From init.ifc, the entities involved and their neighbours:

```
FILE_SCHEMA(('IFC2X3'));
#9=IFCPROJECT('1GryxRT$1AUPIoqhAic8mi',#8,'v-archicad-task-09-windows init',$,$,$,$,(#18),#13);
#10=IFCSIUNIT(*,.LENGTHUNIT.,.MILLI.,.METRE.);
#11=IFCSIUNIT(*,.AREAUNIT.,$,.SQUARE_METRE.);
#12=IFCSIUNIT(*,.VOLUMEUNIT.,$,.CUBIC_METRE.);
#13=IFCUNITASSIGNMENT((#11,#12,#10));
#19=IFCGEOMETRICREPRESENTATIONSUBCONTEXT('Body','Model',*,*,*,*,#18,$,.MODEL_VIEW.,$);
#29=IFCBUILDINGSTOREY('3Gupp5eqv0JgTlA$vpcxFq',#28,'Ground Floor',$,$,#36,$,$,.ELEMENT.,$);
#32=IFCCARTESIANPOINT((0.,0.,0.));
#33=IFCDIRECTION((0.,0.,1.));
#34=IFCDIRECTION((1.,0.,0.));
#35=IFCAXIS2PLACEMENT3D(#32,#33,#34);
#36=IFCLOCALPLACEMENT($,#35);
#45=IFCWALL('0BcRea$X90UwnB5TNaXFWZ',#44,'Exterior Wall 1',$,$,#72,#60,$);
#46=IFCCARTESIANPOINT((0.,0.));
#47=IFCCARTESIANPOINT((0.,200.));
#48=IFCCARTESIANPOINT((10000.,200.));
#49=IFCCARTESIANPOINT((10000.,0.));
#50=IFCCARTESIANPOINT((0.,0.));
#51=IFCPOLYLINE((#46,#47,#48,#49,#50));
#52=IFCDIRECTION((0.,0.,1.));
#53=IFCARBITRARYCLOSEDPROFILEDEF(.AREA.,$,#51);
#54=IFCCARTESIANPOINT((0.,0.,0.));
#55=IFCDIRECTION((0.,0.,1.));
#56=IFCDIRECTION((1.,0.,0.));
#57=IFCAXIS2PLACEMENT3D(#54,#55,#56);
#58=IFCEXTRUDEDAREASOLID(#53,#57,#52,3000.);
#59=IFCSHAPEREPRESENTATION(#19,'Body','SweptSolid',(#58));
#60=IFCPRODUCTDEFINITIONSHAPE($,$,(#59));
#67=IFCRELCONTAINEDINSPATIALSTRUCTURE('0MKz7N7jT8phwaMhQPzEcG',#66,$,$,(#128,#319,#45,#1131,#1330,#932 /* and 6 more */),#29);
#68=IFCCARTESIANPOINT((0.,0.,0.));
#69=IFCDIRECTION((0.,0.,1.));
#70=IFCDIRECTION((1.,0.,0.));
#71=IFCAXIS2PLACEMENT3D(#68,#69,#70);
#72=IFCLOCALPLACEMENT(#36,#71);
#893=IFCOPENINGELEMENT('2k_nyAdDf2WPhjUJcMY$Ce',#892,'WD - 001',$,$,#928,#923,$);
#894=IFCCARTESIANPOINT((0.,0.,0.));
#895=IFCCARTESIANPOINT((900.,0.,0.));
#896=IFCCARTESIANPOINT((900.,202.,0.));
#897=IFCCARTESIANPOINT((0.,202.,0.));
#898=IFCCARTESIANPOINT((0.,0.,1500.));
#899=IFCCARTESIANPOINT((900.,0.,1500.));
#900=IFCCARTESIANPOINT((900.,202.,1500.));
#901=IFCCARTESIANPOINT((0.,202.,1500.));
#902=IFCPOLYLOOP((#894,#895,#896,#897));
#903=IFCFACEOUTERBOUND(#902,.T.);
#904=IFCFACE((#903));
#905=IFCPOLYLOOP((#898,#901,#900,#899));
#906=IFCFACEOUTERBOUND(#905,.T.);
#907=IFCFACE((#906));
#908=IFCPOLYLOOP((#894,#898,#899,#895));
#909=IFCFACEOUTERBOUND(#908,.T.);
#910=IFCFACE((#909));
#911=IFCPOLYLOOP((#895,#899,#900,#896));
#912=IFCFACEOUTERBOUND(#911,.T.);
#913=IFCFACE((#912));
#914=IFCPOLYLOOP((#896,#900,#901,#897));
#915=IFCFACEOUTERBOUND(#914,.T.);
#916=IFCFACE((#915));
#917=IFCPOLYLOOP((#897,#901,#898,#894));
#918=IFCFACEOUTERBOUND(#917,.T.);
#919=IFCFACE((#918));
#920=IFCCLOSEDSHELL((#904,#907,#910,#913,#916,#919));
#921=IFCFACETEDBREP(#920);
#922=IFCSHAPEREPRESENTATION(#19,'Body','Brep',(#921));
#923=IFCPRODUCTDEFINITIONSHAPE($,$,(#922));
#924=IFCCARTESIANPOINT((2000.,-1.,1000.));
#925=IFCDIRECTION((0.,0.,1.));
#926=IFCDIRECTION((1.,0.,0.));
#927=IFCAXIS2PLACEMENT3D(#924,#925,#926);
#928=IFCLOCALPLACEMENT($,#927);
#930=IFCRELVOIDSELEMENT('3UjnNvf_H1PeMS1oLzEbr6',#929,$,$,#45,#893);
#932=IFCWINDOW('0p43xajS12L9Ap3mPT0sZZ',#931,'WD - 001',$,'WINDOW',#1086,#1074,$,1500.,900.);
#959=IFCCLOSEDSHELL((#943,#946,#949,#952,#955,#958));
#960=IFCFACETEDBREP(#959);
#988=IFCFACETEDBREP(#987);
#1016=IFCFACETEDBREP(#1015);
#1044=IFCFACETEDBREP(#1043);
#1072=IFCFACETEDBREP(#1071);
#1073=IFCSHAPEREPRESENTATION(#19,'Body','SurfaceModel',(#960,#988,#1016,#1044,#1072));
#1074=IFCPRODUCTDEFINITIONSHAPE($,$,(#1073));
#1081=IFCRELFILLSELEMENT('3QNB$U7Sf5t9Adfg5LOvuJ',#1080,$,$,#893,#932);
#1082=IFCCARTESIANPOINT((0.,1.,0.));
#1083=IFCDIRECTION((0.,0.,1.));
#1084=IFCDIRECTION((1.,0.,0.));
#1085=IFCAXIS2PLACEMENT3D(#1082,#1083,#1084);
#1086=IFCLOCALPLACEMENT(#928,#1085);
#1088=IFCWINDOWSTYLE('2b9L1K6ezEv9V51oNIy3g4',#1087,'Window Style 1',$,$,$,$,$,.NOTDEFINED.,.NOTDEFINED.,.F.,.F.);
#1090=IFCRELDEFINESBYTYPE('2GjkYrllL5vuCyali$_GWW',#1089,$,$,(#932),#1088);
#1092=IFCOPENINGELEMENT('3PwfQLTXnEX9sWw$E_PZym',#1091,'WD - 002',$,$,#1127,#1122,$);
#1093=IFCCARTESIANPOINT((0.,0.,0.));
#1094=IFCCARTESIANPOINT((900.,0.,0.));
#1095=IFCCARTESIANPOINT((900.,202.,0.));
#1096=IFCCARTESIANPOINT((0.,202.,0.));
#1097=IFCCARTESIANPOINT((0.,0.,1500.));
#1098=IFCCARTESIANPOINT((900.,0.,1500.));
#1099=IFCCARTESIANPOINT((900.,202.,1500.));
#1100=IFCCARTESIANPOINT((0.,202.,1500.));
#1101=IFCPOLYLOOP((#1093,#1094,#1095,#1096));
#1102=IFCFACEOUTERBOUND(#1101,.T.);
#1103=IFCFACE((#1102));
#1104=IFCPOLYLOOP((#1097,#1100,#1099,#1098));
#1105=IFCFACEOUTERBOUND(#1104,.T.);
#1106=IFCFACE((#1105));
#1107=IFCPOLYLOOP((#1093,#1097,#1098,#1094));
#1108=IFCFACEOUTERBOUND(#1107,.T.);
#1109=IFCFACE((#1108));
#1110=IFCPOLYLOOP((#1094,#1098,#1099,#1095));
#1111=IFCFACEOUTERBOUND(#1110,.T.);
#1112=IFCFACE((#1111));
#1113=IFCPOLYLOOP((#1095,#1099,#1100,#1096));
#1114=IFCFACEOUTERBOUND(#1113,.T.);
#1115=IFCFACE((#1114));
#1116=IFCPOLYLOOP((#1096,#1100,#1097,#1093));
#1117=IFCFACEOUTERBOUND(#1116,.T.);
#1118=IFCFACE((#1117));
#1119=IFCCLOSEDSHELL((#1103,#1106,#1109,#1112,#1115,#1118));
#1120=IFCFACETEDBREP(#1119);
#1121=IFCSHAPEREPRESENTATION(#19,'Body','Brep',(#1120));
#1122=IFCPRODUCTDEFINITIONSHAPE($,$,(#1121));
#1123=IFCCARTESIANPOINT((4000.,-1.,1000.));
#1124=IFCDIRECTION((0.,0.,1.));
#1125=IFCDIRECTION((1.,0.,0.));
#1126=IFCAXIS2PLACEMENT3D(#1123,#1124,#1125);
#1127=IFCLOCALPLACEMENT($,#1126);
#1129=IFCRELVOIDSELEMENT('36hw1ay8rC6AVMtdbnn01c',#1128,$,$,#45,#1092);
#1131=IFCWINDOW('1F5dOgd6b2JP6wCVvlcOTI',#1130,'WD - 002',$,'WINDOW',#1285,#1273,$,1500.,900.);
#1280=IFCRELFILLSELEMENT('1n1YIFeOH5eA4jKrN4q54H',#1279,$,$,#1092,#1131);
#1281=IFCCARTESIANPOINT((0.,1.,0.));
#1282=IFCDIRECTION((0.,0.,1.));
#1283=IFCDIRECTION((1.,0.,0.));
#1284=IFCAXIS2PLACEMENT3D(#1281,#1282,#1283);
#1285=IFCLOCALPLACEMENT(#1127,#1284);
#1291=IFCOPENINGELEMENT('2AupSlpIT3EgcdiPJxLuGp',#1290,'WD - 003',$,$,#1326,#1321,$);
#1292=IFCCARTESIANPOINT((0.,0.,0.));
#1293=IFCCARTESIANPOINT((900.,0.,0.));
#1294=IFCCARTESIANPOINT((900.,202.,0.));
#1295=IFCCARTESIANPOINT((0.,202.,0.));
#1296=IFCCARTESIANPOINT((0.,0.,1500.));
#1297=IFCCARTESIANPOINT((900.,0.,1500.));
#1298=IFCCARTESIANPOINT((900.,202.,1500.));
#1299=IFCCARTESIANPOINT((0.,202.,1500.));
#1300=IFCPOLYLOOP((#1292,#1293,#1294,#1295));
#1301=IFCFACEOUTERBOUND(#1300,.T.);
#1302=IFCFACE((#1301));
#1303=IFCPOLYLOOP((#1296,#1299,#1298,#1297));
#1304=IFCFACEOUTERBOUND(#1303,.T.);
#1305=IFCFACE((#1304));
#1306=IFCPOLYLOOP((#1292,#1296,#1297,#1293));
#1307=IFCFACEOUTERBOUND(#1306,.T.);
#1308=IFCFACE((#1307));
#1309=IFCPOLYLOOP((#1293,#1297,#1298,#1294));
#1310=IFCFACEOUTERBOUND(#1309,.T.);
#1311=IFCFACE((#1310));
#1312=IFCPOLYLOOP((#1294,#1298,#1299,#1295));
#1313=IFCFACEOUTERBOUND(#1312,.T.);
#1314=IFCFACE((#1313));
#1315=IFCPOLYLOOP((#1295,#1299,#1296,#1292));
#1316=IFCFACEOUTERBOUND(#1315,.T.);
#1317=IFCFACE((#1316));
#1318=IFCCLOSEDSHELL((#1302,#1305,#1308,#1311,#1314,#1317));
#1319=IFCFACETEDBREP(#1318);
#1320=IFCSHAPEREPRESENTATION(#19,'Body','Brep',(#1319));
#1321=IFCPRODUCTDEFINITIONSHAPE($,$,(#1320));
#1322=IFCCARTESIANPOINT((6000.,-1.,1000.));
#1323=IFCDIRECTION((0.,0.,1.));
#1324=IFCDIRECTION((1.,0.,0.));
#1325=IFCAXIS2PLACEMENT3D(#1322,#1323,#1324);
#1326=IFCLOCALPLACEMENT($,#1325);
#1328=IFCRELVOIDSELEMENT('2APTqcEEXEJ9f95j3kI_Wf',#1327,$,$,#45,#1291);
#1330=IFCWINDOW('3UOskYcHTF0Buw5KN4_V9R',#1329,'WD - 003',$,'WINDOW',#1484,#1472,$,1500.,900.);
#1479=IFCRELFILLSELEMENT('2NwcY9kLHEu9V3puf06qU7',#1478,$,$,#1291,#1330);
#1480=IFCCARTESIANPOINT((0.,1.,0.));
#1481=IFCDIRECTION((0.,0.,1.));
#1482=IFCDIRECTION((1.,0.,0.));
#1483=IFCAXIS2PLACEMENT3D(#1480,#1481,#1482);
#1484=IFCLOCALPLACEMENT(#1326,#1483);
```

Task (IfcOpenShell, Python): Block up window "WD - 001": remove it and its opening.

```python
import ifcopenshell
import ifcopenshell.api.feature
import ifcopenshell.api.root
import ifcopenshell.geom
import ifcopenshell.util.shape

model = ifcopenshell.open("init.ifc")
settings = ifcopenshell.geom.settings()


def volume(element):
    """Net volume in cubic metres, openings subtracted."""
    shape = ifcopenshell.geom.create_shape(settings, element)
    return ifcopenshell.util.shape.get_volume(shape.geometry)


window = model.by_guid("0p43xajS12L9Ap3mPT0sZZ")
opening = window.FillsVoids[0].RelatingOpeningElement
wall = opening.VoidsElements[0].RelatingBuildingElement
before = volume(wall)

ifcopenshell.api.root.remove_product(model, product=window)
ifcopenshell.api.feature.remove_feature(model, feature=opening)

after = volume(wall)

print(f"wall volume {before:.3f} -> {after:.3f} m3")

model.write("init_v2.ifc")
```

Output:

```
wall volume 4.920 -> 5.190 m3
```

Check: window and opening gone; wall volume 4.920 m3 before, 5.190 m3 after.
